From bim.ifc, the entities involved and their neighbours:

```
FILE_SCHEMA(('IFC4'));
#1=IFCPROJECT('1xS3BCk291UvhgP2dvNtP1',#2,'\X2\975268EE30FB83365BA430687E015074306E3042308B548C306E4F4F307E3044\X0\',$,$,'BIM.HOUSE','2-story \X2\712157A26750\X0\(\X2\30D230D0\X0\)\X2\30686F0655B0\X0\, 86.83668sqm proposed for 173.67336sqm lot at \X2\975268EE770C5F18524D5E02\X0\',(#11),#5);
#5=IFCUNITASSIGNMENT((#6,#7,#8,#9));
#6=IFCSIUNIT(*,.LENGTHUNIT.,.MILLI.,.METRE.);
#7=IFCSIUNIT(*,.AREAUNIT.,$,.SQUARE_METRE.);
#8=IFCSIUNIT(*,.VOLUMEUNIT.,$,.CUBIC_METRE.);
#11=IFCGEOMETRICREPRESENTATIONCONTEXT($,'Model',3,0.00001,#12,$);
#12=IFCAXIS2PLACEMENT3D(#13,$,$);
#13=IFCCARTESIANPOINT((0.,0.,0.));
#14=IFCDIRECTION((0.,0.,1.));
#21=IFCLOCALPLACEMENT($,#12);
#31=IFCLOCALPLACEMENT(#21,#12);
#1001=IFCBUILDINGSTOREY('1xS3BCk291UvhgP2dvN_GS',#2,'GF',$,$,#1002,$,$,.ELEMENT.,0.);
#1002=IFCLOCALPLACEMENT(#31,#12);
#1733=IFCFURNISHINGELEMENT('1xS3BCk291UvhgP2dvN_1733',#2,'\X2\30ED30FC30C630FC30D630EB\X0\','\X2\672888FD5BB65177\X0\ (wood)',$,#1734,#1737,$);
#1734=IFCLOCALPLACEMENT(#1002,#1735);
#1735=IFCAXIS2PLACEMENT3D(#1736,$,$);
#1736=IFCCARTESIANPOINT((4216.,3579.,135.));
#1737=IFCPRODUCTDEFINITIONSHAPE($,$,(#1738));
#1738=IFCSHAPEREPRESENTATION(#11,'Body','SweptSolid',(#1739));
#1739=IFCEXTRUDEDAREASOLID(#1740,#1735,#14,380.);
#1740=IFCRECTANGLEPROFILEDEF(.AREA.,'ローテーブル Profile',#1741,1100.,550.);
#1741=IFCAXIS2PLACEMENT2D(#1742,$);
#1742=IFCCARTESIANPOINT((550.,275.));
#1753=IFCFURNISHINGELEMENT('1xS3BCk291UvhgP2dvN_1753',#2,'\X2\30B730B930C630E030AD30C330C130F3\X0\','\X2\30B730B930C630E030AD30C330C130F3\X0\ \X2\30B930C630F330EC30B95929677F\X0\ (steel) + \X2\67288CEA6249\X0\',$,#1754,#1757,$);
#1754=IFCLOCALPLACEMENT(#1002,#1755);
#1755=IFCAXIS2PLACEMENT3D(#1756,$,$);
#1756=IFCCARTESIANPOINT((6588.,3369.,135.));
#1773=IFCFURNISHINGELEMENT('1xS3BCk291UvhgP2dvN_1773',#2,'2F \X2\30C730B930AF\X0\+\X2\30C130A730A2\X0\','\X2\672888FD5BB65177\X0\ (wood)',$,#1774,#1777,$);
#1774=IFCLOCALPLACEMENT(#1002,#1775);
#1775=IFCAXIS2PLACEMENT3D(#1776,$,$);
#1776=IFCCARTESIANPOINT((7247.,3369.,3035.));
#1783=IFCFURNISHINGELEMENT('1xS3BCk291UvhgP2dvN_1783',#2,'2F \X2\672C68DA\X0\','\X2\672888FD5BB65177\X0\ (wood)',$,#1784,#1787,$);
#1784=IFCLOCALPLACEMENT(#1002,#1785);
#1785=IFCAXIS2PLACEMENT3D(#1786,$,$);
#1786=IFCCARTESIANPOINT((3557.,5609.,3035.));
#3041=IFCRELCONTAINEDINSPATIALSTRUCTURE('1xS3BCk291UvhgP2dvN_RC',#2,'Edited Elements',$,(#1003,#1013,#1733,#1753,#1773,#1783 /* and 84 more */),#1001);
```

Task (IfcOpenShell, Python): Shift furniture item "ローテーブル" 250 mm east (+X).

```python
import ifcopenshell
import ifcopenshell.api.geometry
import ifcopenshell.util.placement
import ifcopenshell.util.unit

model = ifcopenshell.open("bim.ifc")
unit_scale = ifcopenshell.util.unit.calculate_unit_scale(model)

item = model.by_guid("1xS3BCk291UvhgP2dvN_1733")
matrix = ifcopenshell.util.placement.get_local_placement(item.ObjectPlacement)
matrix[0, 3] += 0.25 / unit_scale
ifcopenshell.api.geometry.edit_object_placement(model, product=item, matrix=matrix, is_si=False)

print(ifcopenshell.util.placement.get_local_placement(item.ObjectPlacement).round(3) + 0.0)

model.write("bim-out.ifc")
```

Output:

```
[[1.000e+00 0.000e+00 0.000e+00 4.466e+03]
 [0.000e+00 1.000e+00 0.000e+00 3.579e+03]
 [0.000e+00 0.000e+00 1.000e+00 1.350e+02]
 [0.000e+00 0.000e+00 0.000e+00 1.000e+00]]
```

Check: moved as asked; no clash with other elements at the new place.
